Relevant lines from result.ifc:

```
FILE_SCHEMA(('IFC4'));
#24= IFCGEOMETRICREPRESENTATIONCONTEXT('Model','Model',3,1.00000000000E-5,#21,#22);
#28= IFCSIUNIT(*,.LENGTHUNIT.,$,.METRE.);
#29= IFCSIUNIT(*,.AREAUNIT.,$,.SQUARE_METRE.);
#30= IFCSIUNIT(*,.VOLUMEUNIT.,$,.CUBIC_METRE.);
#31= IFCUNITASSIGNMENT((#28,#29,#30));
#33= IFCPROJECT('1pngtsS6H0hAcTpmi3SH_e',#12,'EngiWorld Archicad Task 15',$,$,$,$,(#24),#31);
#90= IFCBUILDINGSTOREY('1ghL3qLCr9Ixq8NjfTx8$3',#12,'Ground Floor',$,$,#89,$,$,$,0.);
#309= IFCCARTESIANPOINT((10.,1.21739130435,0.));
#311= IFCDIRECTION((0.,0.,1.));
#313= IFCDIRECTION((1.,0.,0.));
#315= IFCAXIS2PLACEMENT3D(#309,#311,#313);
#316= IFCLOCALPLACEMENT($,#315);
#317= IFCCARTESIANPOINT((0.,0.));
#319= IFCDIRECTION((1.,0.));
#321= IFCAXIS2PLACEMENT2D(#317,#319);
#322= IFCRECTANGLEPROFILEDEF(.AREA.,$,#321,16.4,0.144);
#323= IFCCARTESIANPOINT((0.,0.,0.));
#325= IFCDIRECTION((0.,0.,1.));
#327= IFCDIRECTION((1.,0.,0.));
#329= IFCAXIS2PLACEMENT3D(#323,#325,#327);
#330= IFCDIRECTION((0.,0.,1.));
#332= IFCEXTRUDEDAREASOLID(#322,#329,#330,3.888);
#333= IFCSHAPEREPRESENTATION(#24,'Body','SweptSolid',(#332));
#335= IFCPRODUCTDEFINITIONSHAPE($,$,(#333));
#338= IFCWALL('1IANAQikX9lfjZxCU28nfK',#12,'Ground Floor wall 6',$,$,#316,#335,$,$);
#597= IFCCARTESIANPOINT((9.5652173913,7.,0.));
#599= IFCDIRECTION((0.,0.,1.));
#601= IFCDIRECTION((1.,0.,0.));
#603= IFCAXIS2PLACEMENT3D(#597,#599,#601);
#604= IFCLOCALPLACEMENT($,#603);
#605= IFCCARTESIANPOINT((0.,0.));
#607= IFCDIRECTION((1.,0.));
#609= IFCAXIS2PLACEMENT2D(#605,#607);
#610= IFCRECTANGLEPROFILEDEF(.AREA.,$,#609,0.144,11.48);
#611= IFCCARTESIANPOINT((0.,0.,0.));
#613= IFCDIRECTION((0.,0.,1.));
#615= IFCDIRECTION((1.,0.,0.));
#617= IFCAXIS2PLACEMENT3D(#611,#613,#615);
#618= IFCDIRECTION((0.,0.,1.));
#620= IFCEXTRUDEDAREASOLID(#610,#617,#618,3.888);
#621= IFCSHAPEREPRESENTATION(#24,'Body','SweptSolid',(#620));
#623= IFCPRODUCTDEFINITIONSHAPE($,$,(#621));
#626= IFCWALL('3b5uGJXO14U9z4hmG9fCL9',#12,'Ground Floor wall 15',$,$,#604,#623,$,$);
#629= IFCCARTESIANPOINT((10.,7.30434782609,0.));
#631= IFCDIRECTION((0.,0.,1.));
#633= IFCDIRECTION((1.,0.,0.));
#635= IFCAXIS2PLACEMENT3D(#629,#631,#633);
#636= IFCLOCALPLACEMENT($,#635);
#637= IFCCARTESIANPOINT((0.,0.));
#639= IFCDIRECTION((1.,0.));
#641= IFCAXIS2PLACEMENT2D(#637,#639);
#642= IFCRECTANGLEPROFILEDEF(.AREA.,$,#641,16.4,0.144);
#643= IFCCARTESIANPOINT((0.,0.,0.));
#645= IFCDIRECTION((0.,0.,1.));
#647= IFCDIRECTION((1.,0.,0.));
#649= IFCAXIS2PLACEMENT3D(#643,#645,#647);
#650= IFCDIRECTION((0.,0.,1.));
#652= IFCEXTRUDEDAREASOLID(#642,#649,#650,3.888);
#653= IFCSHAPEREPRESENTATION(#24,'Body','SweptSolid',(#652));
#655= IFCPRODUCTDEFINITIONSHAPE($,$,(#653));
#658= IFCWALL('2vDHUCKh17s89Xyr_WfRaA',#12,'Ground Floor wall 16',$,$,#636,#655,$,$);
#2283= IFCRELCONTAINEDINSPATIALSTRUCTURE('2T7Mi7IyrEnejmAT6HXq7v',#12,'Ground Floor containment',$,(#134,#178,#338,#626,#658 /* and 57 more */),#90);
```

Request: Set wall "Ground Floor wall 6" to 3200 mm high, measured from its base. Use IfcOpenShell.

```python
import ifcopenshell
import ifcopenshell.geom
import ifcopenshell.util.shape
import ifcopenshell.util.unit

model = ifcopenshell.open("result.ifc")
unit_scale = ifcopenshell.util.unit.calculate_unit_scale(model)
settings = ifcopenshell.geom.settings()


def volume(element):
    """Net volume in cubic metres, openings subtracted."""
    shape = ifcopenshell.geom.create_shape(settings, element)
    return ifcopenshell.util.shape.get_volume(shape.geometry)


wall = model.by_guid("1IANAQikX9lfjZxCU28nfK")
before = volume(wall)

body = next(r for r in wall.Representation.Representations if r.RepresentationIdentifier == "Body")
solid = body.Items[0]
old_height = solid.Depth
solid.Depth = 3.2 / unit_scale
after = volume(wall)

print(f"height {old_height:g} -> {solid.Depth:g}, volume {before:.3f} -> {after:.3f} m3")

model.write("result_updated.ifc")
```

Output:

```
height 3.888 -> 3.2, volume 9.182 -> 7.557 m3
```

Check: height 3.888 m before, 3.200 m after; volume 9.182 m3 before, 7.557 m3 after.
